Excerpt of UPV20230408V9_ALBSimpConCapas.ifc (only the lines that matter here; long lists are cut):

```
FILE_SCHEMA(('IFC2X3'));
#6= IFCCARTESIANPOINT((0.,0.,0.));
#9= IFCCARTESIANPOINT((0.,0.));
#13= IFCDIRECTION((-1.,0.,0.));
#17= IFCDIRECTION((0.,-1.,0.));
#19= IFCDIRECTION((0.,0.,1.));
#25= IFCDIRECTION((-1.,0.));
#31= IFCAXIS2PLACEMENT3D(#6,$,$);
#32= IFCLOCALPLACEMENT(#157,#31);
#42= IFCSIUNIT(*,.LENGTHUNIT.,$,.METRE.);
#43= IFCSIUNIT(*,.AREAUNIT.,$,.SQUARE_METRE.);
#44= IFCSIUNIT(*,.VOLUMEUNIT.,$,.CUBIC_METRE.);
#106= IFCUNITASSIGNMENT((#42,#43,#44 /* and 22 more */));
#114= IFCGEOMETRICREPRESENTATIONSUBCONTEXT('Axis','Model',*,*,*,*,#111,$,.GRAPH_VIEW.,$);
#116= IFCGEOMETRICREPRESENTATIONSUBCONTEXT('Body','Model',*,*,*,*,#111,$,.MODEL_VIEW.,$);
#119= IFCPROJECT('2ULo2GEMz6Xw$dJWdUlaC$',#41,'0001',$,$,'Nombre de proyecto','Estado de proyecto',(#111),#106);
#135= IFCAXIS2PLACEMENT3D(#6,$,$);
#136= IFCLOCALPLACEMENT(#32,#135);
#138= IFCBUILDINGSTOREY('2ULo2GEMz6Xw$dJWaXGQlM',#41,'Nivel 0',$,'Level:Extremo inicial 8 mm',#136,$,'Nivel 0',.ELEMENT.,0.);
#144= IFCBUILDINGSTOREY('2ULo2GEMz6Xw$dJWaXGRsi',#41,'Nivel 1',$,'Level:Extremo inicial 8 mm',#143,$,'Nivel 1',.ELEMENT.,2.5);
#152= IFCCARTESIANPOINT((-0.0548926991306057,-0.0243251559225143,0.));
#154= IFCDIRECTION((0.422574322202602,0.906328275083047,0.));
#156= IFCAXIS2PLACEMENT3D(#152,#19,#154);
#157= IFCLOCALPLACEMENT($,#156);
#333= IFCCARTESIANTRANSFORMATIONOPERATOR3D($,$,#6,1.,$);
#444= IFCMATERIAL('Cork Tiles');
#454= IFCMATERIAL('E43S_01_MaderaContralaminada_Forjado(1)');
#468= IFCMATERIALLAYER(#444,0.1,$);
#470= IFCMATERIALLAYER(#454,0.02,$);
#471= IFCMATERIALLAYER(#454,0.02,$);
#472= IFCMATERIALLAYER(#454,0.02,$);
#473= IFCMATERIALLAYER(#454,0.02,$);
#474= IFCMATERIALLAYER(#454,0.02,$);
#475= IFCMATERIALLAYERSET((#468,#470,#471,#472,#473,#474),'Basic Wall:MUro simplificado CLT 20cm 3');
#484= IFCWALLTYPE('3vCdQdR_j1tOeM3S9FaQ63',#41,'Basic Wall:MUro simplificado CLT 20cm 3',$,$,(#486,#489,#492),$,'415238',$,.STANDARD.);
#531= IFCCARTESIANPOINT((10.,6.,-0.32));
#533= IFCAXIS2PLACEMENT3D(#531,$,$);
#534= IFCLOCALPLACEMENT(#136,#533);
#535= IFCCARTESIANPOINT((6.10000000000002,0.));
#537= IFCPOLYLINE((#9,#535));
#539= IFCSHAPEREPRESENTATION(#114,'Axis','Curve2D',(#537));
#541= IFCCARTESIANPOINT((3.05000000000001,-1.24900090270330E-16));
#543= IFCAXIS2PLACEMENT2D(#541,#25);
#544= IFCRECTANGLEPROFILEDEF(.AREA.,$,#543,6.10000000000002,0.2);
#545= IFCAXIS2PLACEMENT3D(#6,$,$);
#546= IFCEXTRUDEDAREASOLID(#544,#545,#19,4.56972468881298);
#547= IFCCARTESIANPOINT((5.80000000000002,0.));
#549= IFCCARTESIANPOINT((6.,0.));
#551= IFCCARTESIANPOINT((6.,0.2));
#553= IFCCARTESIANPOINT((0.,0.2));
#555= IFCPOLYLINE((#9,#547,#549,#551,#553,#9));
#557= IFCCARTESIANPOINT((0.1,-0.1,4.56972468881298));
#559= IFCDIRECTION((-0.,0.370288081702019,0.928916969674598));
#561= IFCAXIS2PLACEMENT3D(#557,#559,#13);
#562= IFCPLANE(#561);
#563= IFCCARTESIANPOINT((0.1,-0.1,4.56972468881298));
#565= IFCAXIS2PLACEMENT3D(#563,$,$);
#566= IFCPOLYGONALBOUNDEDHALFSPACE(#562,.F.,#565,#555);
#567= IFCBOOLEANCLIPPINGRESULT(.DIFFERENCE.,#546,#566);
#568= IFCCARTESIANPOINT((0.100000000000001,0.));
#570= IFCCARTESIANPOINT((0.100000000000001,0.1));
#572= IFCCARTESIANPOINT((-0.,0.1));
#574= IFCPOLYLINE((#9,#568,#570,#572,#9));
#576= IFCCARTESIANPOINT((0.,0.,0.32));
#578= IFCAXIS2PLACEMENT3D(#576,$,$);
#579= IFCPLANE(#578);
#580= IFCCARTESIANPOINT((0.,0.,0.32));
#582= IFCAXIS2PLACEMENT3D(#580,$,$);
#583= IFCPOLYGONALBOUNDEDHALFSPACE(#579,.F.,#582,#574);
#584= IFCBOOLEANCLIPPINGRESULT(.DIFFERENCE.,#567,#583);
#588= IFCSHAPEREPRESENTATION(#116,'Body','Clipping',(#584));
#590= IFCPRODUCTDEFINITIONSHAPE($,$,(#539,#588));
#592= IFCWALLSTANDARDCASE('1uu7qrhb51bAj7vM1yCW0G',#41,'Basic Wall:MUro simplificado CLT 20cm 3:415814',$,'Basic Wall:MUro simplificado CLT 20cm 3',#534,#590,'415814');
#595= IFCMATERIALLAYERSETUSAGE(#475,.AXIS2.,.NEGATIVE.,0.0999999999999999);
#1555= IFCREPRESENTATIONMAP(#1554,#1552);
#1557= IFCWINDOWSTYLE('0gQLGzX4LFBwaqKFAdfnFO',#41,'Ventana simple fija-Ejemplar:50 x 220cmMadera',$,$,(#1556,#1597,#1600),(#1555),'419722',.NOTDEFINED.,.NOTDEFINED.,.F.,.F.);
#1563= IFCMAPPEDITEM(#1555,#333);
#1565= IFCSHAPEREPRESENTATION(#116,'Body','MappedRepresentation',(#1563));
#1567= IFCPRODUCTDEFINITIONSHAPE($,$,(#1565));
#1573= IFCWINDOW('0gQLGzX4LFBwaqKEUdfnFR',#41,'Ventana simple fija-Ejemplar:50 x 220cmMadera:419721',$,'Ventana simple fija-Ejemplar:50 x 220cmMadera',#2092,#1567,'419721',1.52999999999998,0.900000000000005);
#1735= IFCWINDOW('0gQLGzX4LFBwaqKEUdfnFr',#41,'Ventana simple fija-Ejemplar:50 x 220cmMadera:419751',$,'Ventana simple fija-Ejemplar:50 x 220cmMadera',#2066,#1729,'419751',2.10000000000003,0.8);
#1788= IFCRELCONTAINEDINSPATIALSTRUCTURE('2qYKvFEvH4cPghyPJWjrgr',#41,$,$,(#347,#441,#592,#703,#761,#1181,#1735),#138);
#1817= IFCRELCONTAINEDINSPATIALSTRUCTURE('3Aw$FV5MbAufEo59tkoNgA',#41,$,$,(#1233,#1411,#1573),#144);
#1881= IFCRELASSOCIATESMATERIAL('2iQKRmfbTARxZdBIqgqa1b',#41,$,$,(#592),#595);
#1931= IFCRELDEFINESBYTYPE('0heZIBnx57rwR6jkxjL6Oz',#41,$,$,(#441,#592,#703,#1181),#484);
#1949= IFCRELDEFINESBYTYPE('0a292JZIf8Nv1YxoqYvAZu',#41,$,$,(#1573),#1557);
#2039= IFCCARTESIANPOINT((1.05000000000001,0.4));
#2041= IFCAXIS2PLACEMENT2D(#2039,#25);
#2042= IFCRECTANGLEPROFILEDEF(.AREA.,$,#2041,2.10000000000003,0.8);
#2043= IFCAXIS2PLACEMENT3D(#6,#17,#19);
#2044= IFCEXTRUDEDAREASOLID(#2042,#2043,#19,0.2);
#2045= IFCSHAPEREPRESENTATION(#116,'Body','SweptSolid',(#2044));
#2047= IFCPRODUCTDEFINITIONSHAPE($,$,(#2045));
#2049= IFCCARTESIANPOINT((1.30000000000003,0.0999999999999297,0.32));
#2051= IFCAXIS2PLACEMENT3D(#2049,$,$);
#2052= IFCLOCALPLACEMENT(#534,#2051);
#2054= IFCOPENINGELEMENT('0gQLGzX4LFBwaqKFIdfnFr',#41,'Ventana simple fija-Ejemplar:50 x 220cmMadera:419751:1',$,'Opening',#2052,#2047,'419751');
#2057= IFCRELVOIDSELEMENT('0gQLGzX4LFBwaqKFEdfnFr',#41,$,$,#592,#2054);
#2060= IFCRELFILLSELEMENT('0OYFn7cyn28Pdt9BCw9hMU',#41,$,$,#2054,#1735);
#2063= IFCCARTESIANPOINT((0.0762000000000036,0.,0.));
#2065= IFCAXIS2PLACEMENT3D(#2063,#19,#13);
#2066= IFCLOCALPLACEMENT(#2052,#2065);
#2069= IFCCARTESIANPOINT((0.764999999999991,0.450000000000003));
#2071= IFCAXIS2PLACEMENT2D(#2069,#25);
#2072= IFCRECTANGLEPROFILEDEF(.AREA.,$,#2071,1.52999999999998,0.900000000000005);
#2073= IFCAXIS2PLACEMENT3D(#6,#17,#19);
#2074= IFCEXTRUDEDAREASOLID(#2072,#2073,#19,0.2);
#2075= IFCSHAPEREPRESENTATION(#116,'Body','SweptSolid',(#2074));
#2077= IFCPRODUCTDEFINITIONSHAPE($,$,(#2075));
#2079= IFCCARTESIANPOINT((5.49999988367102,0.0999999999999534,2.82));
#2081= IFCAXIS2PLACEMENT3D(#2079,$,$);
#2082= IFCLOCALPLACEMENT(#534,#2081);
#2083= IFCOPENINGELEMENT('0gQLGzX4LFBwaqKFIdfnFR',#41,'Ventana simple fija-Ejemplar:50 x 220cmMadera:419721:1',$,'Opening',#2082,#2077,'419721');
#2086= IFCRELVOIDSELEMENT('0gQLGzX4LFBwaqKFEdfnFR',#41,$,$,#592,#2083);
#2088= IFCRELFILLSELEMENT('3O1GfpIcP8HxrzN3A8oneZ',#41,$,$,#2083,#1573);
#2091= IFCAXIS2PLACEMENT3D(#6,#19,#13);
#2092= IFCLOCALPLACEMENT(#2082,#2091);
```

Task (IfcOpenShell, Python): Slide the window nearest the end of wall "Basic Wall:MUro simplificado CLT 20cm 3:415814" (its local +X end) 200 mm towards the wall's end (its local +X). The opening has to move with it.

```python
import ifcopenshell
import ifcopenshell.api.geometry
import ifcopenshell.util.placement

model = ifcopenshell.open("UPV20230408V9_ALBSimpConCapas.ifc")

window = model.by_id(1573)
opening = window.FillsVoids[0].RelatingOpeningElement
wall = opening.VoidsElements[0].RelatingBuildingElement

wall_matrix = ifcopenshell.util.placement.get_local_placement(wall.ObjectPlacement)
shift = wall_matrix[:3, 0] * 0.2
before = ifcopenshell.util.placement.get_local_placement(window.ObjectPlacement)[:3, 3].copy()

# The window is placed relative to its opening, so it follows when the opening moves.
matrix = ifcopenshell.util.placement.get_local_placement(opening.ObjectPlacement)
matrix[:3, 3] += shift
ifcopenshell.api.geometry.edit_object_placement(
    model, product=opening, matrix=matrix, is_si=False, should_transform_children=True
)

after = ifcopenshell.util.placement.get_local_placement(window.ObjectPlacement)[:3, 3]
print("window moved by", (after - before).round(3) + 0.0)

model.write("UPV20230408V9_ALBSimpConCapas_v2.ifc")
```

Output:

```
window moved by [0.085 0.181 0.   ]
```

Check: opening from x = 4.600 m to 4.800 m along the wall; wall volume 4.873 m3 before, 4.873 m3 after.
